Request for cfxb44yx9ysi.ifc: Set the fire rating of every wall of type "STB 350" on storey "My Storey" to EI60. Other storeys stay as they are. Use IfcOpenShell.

First a look at what the model holds.

```python
import ifcopenshell
import ifcopenshell.util.element

model = ifcopenshell.open("cfxb44yx9ysi.ifc")
print(model.schema)
storey = next(s for s in model.by_type("IfcBuildingStorey") if s.Name == "My Storey")
walls = [e for e in ifcopenshell.util.element.get_decomposition(storey) if e.is_a("IfcWall")]
seen = {}
for e in walls:
    element_type = ifcopenshell.util.element.get_type(e)
    key = (element_type.Name if element_type != e and element_type else None, ifcopenshell.util.element.get_pset(e, "Pset_WallCommon", "FireRating"))
    seen[key] = seen.get(key, 0) + 1
for (name, value), count in sorted(seen.items(), key=str):
    print(count, "x", name, "|", value)
```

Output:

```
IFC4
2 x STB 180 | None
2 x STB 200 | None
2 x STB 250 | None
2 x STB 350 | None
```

```python
import ifcopenshell
import ifcopenshell.api.pset
import ifcopenshell.util.element

model = ifcopenshell.open("cfxb44yx9ysi.ifc")

storey = next(s for s in model.by_type("IfcBuildingStorey") if s.Name == "My Storey")
walls = [e for e in ifcopenshell.util.element.get_decomposition(storey) if e.is_a("IfcWall")]

count = 0
for e in walls:
    element_type = ifcopenshell.util.element.get_type(e)
    if element_type in (None, e) or element_type.Name != "STB 350":
        continue
    # add_pset returns the element's existing set when there is one.
    pset = ifcopenshell.api.pset.add_pset(model, product=e, name="Pset_WallCommon")
    ifcopenshell.api.pset.edit_pset(model, pset=pset, properties={"FireRating": "EI60"})
    count += 1

print(count, "walls updated")

model.write("cfxb44yx9ysi_updated.ifc")
```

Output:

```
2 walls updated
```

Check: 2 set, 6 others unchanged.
